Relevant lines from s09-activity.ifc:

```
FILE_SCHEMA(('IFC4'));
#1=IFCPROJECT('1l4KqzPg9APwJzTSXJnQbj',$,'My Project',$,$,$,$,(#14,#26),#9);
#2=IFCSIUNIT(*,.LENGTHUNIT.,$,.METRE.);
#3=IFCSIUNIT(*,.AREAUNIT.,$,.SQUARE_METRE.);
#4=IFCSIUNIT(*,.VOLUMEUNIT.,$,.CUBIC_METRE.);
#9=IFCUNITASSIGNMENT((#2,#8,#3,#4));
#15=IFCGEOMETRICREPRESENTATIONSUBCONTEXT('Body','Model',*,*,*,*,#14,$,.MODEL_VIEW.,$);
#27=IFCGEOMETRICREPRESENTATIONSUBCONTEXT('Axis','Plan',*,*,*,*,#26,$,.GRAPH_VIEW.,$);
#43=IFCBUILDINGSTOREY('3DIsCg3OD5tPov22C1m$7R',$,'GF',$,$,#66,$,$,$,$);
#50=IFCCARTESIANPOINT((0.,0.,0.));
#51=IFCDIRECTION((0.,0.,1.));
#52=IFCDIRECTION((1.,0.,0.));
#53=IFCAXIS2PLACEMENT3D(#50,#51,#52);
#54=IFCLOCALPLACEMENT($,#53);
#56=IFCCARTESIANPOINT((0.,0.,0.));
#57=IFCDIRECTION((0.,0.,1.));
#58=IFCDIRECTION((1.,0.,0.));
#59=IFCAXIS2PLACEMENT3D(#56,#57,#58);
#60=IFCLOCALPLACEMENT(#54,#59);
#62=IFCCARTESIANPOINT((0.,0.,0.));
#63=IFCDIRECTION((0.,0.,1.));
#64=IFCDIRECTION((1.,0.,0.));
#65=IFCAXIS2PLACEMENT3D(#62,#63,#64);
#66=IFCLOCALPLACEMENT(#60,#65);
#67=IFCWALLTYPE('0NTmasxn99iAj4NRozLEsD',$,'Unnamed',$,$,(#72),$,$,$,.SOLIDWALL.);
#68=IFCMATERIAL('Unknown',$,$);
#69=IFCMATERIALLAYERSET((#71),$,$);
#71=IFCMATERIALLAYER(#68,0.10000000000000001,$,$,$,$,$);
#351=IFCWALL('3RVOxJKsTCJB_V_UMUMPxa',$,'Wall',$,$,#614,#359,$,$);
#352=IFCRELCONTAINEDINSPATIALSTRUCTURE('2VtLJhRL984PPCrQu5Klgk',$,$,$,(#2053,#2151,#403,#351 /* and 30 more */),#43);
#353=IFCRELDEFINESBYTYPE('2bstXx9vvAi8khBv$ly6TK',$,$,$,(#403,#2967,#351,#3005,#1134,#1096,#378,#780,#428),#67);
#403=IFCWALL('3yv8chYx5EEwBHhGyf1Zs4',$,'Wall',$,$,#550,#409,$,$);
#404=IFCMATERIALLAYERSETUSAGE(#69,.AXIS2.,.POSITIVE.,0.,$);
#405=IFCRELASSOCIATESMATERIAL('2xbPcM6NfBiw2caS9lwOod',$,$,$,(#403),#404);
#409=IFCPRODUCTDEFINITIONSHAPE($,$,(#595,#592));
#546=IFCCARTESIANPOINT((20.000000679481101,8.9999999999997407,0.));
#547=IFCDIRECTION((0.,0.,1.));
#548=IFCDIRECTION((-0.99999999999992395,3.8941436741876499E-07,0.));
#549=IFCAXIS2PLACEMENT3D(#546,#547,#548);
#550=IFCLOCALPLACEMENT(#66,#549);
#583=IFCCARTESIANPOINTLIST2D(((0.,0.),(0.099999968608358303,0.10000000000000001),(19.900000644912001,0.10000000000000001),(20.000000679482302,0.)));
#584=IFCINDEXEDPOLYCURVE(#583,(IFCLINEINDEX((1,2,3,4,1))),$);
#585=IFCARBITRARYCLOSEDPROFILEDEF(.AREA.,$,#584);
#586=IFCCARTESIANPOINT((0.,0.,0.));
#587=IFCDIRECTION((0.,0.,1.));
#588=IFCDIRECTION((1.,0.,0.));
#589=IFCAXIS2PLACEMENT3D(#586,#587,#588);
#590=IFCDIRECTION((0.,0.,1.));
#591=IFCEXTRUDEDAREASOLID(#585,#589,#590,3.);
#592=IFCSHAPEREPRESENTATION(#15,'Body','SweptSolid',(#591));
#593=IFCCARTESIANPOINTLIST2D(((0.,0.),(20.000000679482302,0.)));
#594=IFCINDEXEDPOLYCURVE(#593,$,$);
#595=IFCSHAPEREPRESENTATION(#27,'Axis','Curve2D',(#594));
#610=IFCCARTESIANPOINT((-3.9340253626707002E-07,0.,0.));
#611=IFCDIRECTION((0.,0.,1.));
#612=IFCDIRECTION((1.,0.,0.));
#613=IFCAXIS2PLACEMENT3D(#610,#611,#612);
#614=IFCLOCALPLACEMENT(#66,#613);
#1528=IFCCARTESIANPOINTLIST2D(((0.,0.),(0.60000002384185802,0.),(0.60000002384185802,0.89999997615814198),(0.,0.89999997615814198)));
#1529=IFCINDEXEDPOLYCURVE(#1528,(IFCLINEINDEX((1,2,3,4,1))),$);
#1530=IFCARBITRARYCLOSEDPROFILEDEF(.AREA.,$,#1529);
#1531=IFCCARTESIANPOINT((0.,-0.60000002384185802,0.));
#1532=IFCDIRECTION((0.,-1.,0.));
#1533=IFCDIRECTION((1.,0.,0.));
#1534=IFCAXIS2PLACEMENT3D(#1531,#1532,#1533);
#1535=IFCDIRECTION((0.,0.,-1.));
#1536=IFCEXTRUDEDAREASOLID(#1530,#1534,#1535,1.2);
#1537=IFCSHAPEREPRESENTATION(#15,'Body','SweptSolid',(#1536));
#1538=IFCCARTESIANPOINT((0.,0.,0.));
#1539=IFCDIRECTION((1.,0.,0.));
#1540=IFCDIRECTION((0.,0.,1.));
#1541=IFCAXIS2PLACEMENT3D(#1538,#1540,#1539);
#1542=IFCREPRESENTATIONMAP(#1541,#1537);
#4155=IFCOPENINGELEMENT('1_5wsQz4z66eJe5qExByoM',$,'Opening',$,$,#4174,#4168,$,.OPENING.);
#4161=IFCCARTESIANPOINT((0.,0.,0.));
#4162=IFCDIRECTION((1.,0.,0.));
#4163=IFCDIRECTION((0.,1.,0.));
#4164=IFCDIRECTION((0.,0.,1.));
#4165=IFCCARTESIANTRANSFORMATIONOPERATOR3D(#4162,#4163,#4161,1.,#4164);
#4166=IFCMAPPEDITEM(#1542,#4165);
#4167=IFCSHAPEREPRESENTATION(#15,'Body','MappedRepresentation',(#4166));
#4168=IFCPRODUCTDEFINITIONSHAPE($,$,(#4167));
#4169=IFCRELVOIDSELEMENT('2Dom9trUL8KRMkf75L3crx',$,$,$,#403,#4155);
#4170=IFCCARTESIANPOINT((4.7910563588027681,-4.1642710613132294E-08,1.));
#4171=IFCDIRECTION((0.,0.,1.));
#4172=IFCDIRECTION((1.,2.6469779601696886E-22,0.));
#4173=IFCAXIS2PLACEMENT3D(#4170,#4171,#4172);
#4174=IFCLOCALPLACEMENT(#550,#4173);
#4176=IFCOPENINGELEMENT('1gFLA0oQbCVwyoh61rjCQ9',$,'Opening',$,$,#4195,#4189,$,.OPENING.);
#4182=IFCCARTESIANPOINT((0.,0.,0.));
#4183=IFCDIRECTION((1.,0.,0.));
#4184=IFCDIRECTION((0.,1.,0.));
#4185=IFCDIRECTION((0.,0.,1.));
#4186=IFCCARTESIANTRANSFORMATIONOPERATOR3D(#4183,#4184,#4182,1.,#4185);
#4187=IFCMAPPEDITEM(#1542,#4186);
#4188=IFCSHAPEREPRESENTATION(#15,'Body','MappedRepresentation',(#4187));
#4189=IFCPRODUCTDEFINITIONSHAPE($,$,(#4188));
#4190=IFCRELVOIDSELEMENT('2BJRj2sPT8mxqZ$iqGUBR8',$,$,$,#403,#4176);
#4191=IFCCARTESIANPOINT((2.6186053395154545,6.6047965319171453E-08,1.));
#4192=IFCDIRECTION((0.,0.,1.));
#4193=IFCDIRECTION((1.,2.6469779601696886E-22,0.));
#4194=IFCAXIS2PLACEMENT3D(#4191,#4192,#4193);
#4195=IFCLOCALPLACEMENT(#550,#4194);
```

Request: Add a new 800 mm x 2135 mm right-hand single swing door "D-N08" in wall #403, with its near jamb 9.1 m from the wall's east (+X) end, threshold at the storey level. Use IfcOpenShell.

```python
import numpy as np
import ifcopenshell
import ifcopenshell.api.feature
import ifcopenshell.api.geometry
import ifcopenshell.api.root
import ifcopenshell.api.spatial
import ifcopenshell.geom
import ifcopenshell.util.element
import ifcopenshell.util.placement
import ifcopenshell.util.representation
import ifcopenshell.util.shape
import ifcopenshell.util.unit

model = ifcopenshell.open("s09-activity.ifc")
unit_scale = ifcopenshell.util.unit.calculate_unit_scale(model)
settings = ifcopenshell.geom.settings()


def volume(element):
    """Net volume in cubic metres, openings subtracted."""
    shape = ifcopenshell.geom.create_shape(settings, element)
    return ifcopenshell.util.shape.get_volume(shape.geometry)


wall = model.by_guid("3yv8chYx5EEwBHhGyf1Zs4")
storey = ifcopenshell.util.element.get_container(wall, ifc_class="IfcBuildingStorey")
context = ifcopenshell.util.representation.get_context(model, "Model", "Body", "MODEL_VIEW")
before = volume(wall)

width, height, from_end, sill = 0.8, 2.135, 9.1, 0.0  # metres

# The wall runs along its own X axis, and the end named is its -X end.
wall_shape = ifcopenshell.geom.create_shape(settings, wall)
x, y, z = ifcopenshell.util.shape.get_vertices(wall_shape.geometry).T
start = x.min() + from_end
face, thickness = float(y.min()), float(y.max() - y.min())
wall_matrix = ifcopenshell.util.placement.get_local_placement(wall.ObjectPlacement)
level = ifcopenshell.util.placement.get_local_placement(storey.ObjectPlacement)[2, 3]


def in_wall(x, y):
    """Placement at x, y metres in the wall's axes, at sill height."""
    matrix = wall_matrix.copy()
    matrix[:, 3] = wall_matrix @ np.array([x / unit_scale, y / unit_scale, 0.0, 1.0])
    matrix[2, 3] = level + sill / unit_scale
    return matrix


# Opening: a box that overshoots both wall faces by 50 mm.
opening = ifcopenshell.api.root.create_entity(model, ifc_class="IfcOpeningElement", predefined_type="OPENING")
box = ifcopenshell.api.geometry.add_wall_representation(
    model, context=context, length=width, height=height, thickness=thickness + 0.1
)
ifcopenshell.api.geometry.assign_representation(model, product=opening, representation=box)
ifcopenshell.api.geometry.edit_object_placement(model, product=opening, matrix=in_wall(start, face - 0.05), is_si=False)
ifcopenshell.api.feature.add_feature(model, feature=opening, element=wall)

door = ifcopenshell.api.root.create_entity(model, ifc_class="IfcDoor", name="D-N08", predefined_type="DOOR")
door.OverallWidth, door.OverallHeight = width / unit_scale, height / unit_scale
door.OperationType = "SINGLE_SWING_RIGHT"
body = ifcopenshell.api.geometry.add_door_representation(
    model,
    context=context,
    overall_width=door.OverallWidth,
    overall_height=door.OverallHeight,
    operation_type="SINGLE_SWING_RIGHT",
    lining_properties={"LiningDepth": thickness / unit_scale, "ThresholdDepth": thickness / unit_scale},
)
ifcopenshell.api.geometry.assign_representation(model, product=door, representation=body)
ifcopenshell.api.spatial.assign_container(model, products=[door], relating_structure=storey)
ifcopenshell.api.feature.add_filling(model, opening=opening, element=door)

# The lining spans the wall, so the door starts at the wall face.
ifcopenshell.api.geometry.edit_object_placement(model, product=door, matrix=in_wall(start, face), is_si=False)

after = volume(wall)

print(f"wall volume {before:.3f} -> {after:.3f} m3")

model.write("s09-activity_updated.ifc")
```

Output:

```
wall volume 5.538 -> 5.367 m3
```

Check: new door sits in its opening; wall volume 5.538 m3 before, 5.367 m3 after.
